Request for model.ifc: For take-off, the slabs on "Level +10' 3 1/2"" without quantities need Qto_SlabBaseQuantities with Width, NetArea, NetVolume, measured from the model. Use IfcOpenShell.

First a look at what the model holds.

```python
import ifcopenshell
import ifcopenshell.util.element
import ifcopenshell.util.unit

model = ifcopenshell.open("model.ifc")
print(model.schema)
for unit_type in ("LENGTHUNIT", "AREAUNIT", "VOLUMEUNIT"):
    print(unit_type, ifcopenshell.util.unit.calculate_unit_scale(model, unit_type))
storey = next(s for s in model.by_type("IfcBuildingStorey") if s.Name == 'Level +10\' 3 1/2"')
slabs = [e for e in ifcopenshell.util.element.get_decomposition(storey) if e.is_a("IfcSlab")]
for e in sorted(slabs, key=lambda e: e.id()):
    print(e.id(), e.is_a(), e.Name, list(ifcopenshell.util.element.get_psets(e, qtos_only=True)), sep=" | ")
```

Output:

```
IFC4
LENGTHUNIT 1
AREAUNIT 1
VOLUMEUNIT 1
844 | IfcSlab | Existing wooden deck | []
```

```python
import ifcopenshell
import ifcopenshell.api.pset
import ifcopenshell.geom
import ifcopenshell.util.element
import ifcopenshell.util.shape
import ifcopenshell.util.unit

model = ifcopenshell.open("model.ifc")
unit_scale = ifcopenshell.util.unit.calculate_unit_scale(model)
area_scale = ifcopenshell.util.unit.calculate_unit_scale(model, "AREAUNIT")
volume_scale = ifcopenshell.util.unit.calculate_unit_scale(model, "VOLUMEUNIT")
settings = ifcopenshell.geom.settings()

storey = next(s for s in model.by_type("IfcBuildingStorey") if s.Name == 'Level +10\' 3 1/2"')
slabs = [e for e in ifcopenshell.util.element.get_decomposition(storey) if e.is_a("IfcSlab")]

for e in sorted(slabs, key=lambda e: e.id()):
    if ifcopenshell.util.element.get_psets(e, qtos_only=True, should_inherit=False):
        continue
    # Geometry comes back in metres, in the element's own axes.
    shape = ifcopenshell.geom.create_shape(settings, e)
    values = {
        "Width": ifcopenshell.util.shape.get_z(shape.geometry) / unit_scale,
        "NetArea": ifcopenshell.util.shape.get_footprint_area(shape.geometry) / area_scale,
        "NetVolume": ifcopenshell.util.shape.get_volume(shape.geometry) / volume_scale,
    }
    qto = ifcopenshell.api.pset.add_qto(model, product=e, name="Qto_SlabBaseQuantities")
    ifcopenshell.api.pset.edit_qto(model, qto=qto, properties=values)
    print(e.id(), {k: round(v, 3) for k, v in values.items()})

model.write("model-out.ifc")
```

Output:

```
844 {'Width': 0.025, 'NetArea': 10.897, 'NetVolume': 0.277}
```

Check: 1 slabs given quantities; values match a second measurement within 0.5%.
